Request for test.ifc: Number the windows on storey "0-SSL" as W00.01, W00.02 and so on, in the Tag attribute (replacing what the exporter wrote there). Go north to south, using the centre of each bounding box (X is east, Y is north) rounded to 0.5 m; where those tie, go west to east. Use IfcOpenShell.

First a look at what the model holds.

```python
import ifcopenshell
import ifcopenshell.util.element
import ifcopenshell.util.placement

model = ifcopenshell.open("test.ifc")
print(model.schema)
storey = next(s for s in model.by_type("IfcBuildingStorey") if s.Name == "0-SSL")
windows = [e for e in ifcopenshell.util.element.get_decomposition(storey) if e.is_a("IfcWindow")]
for e in sorted(windows, key=lambda e: e.id()):
    origin = ifcopenshell.util.placement.get_local_placement(e.ObjectPlacement)[:3, 3]
    print(e.id(), e.Tag, e.Name, origin.round(2) + 0.0, sep=" | ")
```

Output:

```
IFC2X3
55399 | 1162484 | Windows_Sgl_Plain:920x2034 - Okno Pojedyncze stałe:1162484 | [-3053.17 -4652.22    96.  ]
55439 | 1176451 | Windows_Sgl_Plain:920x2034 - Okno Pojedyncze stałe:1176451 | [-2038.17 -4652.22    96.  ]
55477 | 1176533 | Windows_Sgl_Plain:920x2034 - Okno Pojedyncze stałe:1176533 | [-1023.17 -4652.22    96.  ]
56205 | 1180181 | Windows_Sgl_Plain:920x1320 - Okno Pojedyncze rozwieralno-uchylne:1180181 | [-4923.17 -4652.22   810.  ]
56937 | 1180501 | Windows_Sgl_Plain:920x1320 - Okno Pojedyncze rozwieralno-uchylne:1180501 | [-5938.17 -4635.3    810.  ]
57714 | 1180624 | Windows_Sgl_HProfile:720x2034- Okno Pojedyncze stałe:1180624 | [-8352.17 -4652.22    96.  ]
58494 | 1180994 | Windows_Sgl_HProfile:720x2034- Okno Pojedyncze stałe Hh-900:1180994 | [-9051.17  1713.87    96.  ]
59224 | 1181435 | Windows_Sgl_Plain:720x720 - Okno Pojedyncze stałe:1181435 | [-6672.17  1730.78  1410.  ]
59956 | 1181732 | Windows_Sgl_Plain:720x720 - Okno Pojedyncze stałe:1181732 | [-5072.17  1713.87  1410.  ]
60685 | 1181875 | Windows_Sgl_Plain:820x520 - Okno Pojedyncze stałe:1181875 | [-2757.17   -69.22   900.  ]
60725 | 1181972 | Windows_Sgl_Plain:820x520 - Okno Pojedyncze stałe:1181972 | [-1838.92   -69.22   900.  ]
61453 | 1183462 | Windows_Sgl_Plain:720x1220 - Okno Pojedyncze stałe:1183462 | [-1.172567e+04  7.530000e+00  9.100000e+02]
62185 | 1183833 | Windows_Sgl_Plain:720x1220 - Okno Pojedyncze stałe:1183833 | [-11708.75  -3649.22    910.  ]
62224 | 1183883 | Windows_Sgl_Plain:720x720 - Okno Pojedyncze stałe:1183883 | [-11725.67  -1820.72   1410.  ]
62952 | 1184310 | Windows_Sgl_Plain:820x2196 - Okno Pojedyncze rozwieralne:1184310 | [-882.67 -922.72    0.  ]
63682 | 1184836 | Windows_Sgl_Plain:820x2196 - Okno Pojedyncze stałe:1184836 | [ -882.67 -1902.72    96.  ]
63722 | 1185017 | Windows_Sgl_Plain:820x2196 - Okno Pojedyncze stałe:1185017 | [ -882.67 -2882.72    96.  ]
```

```python
import ifcopenshell
import ifcopenshell.geom
import ifcopenshell.util.element
import ifcopenshell.util.shape

model = ifcopenshell.open("test.ifc")
settings = ifcopenshell.geom.settings()
settings.set("use-world-coords", True)


def centre(element):
    shape = ifcopenshell.geom.create_shape(settings, element)
    return ifcopenshell.util.shape.get_bbox_centroid(shape.geometry)


storey = next(s for s in model.by_type("IfcBuildingStorey") if s.Name == "0-SSL")
windows = [e for e in ifcopenshell.util.element.get_decomposition(storey) if e.is_a("IfcWindow")]

# Insertion points can sit at a corner or the storey origin, so sort by the geometry (in metres).
centres = {e: centre(e) for e in windows}
windows.sort(key=lambda e: (-round(centres[e][1] / 0.5), centres[e][0]))

for i, e in enumerate(windows, start=1):
    number = f"W00.{i:02d}"
    e.Tag = number
    print(e.id(), number)

model.write("test_v2.ifc")
```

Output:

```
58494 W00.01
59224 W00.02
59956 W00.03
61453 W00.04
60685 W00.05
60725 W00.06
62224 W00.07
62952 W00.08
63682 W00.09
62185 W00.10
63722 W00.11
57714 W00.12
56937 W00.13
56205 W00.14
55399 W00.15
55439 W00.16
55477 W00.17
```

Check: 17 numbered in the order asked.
